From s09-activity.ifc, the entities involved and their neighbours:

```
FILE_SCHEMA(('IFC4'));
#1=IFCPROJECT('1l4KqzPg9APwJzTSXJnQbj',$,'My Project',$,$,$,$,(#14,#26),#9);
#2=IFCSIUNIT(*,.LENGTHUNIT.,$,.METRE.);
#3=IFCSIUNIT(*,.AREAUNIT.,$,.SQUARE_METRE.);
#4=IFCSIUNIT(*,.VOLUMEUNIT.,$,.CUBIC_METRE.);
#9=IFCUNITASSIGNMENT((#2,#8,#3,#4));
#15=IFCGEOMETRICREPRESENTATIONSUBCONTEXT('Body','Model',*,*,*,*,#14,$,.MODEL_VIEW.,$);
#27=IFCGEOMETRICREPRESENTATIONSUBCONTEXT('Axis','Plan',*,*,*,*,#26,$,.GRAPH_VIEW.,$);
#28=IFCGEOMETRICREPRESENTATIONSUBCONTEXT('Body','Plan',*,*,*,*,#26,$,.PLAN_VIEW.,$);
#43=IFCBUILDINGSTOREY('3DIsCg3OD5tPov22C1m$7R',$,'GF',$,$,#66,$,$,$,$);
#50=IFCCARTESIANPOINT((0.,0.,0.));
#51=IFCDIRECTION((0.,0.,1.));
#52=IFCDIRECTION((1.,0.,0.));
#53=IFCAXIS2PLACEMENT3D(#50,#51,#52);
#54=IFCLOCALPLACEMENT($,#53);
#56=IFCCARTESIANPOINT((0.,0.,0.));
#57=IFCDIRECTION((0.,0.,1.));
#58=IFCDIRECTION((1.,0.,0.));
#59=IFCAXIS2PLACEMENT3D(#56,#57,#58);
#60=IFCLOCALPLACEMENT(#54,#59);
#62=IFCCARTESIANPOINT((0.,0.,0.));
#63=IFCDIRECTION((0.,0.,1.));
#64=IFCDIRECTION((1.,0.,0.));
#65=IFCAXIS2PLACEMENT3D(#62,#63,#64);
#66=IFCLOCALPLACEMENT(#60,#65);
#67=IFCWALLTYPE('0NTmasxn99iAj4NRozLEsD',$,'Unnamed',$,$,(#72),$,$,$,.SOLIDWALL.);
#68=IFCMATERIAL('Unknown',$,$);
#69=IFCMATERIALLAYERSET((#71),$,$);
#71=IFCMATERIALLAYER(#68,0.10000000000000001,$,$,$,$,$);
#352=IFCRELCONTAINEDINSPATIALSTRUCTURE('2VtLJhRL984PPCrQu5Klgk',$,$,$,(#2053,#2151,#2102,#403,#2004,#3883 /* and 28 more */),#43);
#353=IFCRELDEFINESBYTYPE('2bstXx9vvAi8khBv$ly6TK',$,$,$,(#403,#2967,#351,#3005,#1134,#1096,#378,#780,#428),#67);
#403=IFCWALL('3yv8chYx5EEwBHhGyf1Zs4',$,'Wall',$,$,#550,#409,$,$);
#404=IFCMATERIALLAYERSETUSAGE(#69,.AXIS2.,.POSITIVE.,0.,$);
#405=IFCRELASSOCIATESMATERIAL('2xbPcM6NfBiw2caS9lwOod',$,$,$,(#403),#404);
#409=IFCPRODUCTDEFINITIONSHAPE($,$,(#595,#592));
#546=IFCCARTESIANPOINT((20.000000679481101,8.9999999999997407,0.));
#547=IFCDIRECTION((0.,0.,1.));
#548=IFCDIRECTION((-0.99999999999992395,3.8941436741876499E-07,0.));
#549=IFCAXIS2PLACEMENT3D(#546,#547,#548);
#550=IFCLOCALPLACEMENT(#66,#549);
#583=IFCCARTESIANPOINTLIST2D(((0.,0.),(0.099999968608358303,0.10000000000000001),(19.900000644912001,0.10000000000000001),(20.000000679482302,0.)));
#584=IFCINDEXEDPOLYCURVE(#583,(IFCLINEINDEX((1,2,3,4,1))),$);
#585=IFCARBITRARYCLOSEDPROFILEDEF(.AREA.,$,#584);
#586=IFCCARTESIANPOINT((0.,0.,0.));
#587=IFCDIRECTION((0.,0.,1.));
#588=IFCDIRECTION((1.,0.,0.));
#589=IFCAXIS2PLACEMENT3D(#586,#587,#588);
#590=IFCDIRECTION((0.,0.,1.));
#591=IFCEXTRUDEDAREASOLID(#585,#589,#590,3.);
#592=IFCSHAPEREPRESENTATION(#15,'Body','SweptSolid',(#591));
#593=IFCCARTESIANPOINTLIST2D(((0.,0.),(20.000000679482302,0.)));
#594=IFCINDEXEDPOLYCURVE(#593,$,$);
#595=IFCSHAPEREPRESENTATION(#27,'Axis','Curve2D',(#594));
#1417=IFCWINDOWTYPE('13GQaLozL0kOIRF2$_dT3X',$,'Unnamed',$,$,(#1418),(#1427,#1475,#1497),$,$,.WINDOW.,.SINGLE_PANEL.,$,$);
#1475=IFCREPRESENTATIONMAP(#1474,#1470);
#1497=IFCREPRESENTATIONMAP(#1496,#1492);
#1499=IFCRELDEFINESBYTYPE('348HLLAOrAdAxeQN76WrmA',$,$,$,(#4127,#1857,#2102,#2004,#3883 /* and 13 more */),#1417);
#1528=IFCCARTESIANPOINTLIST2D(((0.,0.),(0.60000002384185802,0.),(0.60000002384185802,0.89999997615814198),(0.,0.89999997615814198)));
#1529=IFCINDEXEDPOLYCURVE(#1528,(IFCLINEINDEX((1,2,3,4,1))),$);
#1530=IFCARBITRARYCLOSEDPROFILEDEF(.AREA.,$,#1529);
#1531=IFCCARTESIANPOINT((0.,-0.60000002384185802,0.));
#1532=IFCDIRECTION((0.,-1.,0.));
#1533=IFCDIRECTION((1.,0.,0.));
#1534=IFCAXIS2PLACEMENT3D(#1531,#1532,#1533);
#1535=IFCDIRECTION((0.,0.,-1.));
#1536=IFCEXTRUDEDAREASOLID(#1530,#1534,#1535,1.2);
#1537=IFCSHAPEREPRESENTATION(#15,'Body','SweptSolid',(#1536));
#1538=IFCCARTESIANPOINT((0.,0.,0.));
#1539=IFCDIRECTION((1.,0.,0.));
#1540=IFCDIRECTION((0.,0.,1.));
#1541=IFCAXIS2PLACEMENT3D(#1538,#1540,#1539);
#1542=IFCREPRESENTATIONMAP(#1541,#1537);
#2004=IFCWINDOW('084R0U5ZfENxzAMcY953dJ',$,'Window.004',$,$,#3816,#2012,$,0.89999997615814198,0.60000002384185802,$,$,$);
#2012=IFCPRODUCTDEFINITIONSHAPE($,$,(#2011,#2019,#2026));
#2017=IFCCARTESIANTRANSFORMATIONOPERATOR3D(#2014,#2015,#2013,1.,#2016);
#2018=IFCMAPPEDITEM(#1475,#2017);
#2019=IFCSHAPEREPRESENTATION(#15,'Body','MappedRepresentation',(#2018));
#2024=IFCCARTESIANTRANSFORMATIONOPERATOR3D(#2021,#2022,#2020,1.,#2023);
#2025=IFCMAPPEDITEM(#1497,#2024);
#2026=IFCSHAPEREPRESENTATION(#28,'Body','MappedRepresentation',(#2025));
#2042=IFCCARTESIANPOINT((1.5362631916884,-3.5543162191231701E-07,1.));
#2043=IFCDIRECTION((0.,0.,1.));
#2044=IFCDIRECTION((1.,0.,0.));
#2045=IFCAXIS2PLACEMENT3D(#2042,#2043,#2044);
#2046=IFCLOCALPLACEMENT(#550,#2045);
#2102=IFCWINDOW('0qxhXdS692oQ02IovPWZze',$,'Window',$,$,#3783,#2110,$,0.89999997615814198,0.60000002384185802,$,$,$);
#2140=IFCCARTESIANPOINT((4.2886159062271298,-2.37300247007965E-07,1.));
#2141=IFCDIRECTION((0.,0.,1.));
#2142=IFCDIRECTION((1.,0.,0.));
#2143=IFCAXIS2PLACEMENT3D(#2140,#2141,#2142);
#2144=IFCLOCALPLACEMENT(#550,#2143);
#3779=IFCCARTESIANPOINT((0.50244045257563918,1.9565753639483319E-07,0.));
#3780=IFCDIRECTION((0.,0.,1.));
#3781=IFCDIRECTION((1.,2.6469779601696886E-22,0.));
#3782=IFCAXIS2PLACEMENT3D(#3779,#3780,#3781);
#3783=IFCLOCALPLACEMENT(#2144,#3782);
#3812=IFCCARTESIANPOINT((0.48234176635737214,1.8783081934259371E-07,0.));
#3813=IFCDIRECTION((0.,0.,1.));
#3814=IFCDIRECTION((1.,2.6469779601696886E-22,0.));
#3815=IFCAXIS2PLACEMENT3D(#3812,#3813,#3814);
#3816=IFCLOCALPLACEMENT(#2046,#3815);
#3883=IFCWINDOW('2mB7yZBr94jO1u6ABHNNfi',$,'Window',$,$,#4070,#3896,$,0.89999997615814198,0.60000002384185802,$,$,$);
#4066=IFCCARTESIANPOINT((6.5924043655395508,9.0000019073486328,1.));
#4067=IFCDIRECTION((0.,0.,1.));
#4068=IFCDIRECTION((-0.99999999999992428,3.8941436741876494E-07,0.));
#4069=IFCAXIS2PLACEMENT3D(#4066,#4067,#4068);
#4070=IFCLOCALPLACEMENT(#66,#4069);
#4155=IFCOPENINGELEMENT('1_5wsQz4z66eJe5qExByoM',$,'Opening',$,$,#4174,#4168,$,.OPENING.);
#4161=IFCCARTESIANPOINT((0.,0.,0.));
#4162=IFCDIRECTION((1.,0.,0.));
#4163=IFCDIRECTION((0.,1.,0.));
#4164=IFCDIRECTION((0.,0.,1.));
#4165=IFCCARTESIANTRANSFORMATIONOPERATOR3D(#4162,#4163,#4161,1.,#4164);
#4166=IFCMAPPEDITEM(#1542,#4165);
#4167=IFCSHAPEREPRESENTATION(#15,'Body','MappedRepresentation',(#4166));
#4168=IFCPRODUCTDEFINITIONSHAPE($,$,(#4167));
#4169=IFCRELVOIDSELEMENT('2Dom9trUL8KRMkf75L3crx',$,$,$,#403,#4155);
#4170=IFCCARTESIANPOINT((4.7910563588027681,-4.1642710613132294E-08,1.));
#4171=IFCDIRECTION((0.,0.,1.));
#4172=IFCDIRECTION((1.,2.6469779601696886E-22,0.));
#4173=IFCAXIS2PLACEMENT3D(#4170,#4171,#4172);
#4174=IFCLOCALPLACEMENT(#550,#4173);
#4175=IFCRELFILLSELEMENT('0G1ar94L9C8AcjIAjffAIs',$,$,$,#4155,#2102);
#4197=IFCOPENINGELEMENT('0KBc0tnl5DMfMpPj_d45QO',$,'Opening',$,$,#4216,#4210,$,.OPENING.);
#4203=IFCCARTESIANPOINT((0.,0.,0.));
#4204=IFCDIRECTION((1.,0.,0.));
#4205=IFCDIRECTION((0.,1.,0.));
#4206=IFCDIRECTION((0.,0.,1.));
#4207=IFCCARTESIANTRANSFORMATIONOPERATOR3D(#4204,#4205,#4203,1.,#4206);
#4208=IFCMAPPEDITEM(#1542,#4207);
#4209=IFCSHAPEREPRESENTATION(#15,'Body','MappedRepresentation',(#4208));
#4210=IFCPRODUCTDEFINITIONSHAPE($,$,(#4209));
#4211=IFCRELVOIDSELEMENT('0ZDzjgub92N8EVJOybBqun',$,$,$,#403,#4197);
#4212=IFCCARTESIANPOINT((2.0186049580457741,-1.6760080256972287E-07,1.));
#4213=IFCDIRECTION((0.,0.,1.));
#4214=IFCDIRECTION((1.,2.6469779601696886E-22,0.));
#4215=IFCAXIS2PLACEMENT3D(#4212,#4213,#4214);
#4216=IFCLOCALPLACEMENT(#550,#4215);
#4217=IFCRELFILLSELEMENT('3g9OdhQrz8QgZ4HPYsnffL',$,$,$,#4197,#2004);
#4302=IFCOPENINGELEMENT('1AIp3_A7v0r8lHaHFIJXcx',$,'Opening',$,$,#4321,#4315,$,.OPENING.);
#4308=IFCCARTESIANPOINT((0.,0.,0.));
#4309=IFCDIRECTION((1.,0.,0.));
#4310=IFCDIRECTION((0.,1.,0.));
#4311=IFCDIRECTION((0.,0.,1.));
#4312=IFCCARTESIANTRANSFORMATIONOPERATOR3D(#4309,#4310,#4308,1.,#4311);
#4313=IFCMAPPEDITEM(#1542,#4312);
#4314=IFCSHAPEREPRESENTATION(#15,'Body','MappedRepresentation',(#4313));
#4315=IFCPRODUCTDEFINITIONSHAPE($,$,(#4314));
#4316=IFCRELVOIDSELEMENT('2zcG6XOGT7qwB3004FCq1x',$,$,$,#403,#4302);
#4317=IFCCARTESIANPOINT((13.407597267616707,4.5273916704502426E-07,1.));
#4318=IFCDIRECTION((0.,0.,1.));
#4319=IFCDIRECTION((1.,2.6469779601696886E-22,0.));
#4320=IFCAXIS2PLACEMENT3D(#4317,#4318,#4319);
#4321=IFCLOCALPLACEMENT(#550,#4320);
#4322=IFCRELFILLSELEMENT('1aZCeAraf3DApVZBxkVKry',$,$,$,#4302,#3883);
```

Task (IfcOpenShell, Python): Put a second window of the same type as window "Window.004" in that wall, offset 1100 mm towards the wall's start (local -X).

```python
import ifcopenshell
import ifcopenshell.api.feature
import ifcopenshell.api.geometry
import ifcopenshell.api.root
import ifcopenshell.geom
import ifcopenshell.util.element
import ifcopenshell.util.placement
import ifcopenshell.util.shape
import ifcopenshell.util.unit

model = ifcopenshell.open("s09-activity.ifc")
unit_scale = ifcopenshell.util.unit.calculate_unit_scale(model)
settings = ifcopenshell.geom.settings()


def volume(element):
    """Net volume in cubic metres, openings subtracted."""
    shape = ifcopenshell.geom.create_shape(settings, element)
    return ifcopenshell.util.shape.get_volume(shape.geometry)


window = model.by_id(2004)
opening = window.FillsVoids[0].RelatingOpeningElement
wall = opening.VoidsElements[0].RelatingBuildingElement
before = volume(wall)
shift = ifcopenshell.util.placement.get_local_placement(wall.ObjectPlacement)[:3, 0] * -1.1 / unit_scale

# copy_class copies the void relationship, type, container and properties, but no geometry.
new_opening = ifcopenshell.api.root.copy_class(model, product=opening)
new_opening.Representation = ifcopenshell.util.element.copy_deep(
    model, opening.Representation, exclude=["IfcGeometricRepresentationContext", "IfcRepresentationMap"]
)
new_window = ifcopenshell.api.root.copy_class(model, product=window)
new_window.Representation = ifcopenshell.util.element.copy_deep(
    model, window.Representation, exclude=["IfcGeometricRepresentationContext", "IfcRepresentationMap"]
)
ifcopenshell.api.feature.add_filling(model, opening=new_opening, element=new_window)

for old, new in ((opening, new_opening), (window, new_window)):
    matrix = ifcopenshell.util.placement.get_local_placement(old.ObjectPlacement)
    matrix[:3, 3] += shift
    ifcopenshell.api.geometry.edit_object_placement(model, product=new, matrix=matrix, is_si=False)

after = volume(wall)

print(f"wall volume {before:.3f} -> {after:.3f} m3")

model.write("s09-activity_updated.ifc")
```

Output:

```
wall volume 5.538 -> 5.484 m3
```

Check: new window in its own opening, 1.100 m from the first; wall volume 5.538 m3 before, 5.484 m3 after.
